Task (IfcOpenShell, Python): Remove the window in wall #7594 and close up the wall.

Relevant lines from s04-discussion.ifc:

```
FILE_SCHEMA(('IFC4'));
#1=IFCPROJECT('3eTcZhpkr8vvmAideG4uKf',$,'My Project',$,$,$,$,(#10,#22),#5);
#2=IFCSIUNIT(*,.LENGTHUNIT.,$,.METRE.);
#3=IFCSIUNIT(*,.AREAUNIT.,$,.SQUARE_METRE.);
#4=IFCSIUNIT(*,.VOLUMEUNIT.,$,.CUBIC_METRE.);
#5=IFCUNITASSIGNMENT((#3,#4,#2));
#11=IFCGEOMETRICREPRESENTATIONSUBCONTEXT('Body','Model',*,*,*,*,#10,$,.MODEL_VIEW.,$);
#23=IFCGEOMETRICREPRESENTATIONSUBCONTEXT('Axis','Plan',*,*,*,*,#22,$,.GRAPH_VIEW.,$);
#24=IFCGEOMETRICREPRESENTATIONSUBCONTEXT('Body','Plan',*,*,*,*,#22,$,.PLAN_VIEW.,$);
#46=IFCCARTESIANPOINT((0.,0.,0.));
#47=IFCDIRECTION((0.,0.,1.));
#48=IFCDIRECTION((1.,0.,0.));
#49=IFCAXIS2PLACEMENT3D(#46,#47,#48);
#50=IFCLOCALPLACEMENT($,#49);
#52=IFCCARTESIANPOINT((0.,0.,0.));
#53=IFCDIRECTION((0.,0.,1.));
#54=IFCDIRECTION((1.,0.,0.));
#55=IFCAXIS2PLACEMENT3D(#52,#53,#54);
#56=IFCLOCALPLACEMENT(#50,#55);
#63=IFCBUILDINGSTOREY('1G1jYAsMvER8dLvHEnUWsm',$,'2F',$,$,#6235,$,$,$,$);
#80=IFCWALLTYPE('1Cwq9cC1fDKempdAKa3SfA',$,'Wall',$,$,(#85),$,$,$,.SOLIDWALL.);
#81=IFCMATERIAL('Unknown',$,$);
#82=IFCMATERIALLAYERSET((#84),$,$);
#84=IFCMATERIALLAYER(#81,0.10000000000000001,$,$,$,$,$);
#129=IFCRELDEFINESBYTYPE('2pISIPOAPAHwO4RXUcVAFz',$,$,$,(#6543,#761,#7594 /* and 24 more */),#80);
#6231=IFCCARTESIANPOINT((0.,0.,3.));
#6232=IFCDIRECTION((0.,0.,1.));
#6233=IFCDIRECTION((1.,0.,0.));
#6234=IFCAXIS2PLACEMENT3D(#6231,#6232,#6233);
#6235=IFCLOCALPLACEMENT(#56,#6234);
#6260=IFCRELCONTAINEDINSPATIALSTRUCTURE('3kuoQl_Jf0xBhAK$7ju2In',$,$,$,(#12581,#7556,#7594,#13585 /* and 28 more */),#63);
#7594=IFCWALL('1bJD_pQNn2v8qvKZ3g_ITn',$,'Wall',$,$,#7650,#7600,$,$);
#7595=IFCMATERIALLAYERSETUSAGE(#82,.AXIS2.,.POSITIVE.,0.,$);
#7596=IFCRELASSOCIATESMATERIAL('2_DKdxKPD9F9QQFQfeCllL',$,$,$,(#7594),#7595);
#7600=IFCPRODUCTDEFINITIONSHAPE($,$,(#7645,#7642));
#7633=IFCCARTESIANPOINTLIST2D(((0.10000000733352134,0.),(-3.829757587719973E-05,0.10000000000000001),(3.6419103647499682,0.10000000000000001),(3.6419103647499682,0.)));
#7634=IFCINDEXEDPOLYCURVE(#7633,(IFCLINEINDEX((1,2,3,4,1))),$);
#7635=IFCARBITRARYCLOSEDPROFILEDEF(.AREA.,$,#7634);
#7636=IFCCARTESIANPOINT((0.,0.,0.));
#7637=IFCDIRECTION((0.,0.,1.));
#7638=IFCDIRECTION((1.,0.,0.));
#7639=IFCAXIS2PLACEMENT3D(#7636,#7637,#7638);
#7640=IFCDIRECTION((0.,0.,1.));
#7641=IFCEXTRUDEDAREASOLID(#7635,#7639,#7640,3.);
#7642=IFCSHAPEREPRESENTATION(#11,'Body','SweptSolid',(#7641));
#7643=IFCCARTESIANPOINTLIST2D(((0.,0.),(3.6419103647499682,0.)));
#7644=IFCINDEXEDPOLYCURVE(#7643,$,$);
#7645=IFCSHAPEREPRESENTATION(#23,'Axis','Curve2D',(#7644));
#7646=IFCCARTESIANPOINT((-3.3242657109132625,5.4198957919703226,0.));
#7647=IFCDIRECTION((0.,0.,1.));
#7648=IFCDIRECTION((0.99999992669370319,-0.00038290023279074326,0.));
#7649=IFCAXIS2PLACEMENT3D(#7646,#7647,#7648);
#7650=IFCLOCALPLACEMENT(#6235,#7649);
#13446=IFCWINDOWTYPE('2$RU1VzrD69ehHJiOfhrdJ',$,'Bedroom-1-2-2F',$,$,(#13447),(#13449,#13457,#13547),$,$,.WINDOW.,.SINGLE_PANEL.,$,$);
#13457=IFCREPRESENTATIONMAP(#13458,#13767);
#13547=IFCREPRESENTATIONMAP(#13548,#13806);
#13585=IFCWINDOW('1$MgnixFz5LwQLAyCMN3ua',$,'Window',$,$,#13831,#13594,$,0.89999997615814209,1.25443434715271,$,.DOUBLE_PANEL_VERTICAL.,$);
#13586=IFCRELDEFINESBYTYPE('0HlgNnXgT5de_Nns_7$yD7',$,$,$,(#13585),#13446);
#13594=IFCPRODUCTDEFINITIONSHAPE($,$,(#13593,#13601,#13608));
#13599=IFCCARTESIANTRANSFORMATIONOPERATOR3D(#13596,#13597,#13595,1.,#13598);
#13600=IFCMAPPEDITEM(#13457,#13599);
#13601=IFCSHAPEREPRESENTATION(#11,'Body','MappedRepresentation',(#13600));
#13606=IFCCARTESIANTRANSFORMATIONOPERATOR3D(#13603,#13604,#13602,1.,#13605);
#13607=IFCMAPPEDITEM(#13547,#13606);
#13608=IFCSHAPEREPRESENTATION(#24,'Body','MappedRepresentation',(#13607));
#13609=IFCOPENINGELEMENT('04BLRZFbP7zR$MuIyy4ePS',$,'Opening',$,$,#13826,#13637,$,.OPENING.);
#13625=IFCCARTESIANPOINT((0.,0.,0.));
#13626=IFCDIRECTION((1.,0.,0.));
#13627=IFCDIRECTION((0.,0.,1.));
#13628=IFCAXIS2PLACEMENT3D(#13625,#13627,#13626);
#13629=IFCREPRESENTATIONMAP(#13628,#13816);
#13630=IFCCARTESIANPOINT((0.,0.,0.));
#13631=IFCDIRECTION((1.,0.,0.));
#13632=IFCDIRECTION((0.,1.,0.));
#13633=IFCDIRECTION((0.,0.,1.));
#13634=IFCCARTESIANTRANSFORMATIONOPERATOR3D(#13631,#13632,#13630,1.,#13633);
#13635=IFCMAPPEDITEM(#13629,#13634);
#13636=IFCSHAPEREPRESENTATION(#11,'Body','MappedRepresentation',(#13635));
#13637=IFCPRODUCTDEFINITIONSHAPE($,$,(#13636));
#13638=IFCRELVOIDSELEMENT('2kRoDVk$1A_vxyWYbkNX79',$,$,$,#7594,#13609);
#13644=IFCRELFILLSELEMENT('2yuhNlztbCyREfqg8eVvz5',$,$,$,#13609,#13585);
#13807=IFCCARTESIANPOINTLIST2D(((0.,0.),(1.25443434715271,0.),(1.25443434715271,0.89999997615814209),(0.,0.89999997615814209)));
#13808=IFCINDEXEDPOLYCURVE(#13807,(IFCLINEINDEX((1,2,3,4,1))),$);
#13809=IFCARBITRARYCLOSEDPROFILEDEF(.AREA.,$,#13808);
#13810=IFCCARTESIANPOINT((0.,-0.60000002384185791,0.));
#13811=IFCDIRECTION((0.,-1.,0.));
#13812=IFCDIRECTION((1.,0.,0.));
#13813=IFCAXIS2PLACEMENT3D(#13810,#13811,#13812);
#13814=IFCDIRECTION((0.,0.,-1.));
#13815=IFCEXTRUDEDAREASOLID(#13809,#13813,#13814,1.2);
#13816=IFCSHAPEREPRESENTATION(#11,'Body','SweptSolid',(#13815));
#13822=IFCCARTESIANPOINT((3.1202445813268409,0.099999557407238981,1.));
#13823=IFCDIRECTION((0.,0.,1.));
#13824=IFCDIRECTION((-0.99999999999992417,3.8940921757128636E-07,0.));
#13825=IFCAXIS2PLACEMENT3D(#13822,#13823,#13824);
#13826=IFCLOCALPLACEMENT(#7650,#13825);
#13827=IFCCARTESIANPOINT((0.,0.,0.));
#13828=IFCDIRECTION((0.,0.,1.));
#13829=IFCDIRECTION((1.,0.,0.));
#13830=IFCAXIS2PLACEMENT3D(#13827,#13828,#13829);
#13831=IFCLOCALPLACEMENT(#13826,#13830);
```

```python
import ifcopenshell
import ifcopenshell.api.feature
import ifcopenshell.api.root
import ifcopenshell.geom
import ifcopenshell.util.shape

model = ifcopenshell.open("s04-discussion.ifc")
settings = ifcopenshell.geom.settings()


def volume(element):
    """Net volume in cubic metres, openings subtracted."""
    shape = ifcopenshell.geom.create_shape(settings, element)
    return ifcopenshell.util.shape.get_volume(shape.geometry)


window = model.by_id(13585)
opening = window.FillsVoids[0].RelatingOpeningElement
wall = opening.VoidsElements[0].RelatingBuildingElement
before = volume(wall)

ifcopenshell.api.root.remove_product(model, product=window)
ifcopenshell.api.feature.remove_feature(model, feature=opening)

after = volume(wall)

print(f"wall volume {before:.3f} -> {after:.3f} m3")

model.write("s04-discussion_updated.ifc")
```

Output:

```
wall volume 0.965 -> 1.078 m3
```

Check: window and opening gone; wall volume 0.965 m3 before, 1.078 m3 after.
